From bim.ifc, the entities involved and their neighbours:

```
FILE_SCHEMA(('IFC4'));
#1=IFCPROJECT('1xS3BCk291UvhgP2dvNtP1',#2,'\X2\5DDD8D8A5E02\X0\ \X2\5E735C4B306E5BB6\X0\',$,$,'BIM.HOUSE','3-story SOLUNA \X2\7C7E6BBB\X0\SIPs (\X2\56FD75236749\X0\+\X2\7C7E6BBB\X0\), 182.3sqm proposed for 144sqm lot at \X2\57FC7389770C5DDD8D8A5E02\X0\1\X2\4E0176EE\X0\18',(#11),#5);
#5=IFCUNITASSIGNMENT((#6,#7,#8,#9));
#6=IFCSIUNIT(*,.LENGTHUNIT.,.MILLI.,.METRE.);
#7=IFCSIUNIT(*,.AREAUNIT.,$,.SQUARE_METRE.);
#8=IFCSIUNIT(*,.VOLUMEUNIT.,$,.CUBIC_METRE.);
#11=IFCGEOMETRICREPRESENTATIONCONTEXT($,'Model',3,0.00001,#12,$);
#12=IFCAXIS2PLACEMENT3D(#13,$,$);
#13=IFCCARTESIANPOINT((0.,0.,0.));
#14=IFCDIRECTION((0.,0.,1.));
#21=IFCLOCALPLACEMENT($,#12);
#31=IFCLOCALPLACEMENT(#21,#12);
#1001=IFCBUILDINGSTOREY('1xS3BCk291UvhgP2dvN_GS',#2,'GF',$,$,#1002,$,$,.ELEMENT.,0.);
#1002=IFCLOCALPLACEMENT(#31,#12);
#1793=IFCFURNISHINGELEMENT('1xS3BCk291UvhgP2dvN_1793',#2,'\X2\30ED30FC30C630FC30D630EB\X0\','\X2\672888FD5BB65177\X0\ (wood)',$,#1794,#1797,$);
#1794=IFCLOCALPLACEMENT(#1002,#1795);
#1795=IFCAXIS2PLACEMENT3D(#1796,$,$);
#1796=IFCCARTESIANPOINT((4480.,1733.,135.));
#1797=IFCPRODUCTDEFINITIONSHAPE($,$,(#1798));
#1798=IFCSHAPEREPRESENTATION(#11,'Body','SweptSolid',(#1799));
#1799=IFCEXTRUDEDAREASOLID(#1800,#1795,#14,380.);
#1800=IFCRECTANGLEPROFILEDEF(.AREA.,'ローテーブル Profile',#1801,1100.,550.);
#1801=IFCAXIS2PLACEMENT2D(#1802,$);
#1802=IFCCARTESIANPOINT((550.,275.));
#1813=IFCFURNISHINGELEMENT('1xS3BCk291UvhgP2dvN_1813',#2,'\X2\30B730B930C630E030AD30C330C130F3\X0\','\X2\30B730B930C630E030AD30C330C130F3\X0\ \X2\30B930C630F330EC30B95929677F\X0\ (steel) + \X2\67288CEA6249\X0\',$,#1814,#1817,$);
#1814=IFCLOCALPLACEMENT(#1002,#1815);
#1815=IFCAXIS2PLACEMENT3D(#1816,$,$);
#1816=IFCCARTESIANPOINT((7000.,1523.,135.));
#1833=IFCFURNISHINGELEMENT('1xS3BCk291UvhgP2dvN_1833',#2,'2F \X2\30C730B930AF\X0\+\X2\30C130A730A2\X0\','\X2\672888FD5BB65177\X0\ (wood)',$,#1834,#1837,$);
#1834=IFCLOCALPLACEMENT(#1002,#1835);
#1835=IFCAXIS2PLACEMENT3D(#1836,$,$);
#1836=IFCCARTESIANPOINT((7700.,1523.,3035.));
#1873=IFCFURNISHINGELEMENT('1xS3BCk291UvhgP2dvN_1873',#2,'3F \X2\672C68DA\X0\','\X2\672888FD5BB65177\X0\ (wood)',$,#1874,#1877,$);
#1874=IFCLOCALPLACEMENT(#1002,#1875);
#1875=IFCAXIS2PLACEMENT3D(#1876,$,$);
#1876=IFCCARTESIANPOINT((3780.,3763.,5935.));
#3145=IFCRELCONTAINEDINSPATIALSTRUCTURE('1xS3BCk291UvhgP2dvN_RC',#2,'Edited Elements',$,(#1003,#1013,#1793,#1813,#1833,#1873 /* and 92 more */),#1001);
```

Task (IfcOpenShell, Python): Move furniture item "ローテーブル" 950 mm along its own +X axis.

```python
import ifcopenshell
import ifcopenshell.api.geometry
import ifcopenshell.util.placement
import ifcopenshell.util.unit

model = ifcopenshell.open("bim.ifc")
unit_scale = ifcopenshell.util.unit.calculate_unit_scale(model)

item = model.by_guid("1xS3BCk291UvhgP2dvN_1793")
matrix = ifcopenshell.util.placement.get_local_placement(item.ObjectPlacement)
matrix[:3, 3] += matrix[:3, 0] * 0.95 / unit_scale
ifcopenshell.api.geometry.edit_object_placement(model, product=item, matrix=matrix, is_si=False)

print(ifcopenshell.util.placement.get_local_placement(item.ObjectPlacement).round(3) + 0.0)

model.write("bim-out.ifc")
```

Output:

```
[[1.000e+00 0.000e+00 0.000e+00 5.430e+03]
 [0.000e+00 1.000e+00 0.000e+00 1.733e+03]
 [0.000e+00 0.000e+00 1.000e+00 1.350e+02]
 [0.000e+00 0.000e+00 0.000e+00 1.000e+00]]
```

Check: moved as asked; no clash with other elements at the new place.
